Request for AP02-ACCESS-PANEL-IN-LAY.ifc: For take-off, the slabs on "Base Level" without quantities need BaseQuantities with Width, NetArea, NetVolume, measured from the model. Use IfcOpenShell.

First a look at what the model holds.

```python
import ifcopenshell
import ifcopenshell.util.element
import ifcopenshell.util.unit

model = ifcopenshell.open("AP02-ACCESS-PANEL-IN-LAY.ifc")
print(model.schema)
for unit_type in ("LENGTHUNIT", "AREAUNIT", "VOLUMEUNIT"):
    print(unit_type, ifcopenshell.util.unit.calculate_unit_scale(model, unit_type))
storey = next(s for s in model.by_type("IfcBuildingStorey") if s.Name == "Base Level")
slabs = [e for e in ifcopenshell.util.element.get_decomposition(storey) if e.is_a("IfcSlab")]
for e in sorted(slabs, key=lambda e: e.id()):
    print(e.id(), e.is_a(), e.Name, list(ifcopenshell.util.element.get_psets(e, qtos_only=True)), sep=" | ")
```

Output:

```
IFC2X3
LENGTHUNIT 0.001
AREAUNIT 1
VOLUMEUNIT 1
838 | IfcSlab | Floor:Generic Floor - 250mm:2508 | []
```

```python
import ifcopenshell
import ifcopenshell.api.pset
import ifcopenshell.geom
import ifcopenshell.util.element
import ifcopenshell.util.shape
import ifcopenshell.util.unit

model = ifcopenshell.open("AP02-ACCESS-PANEL-IN-LAY.ifc")
unit_scale = ifcopenshell.util.unit.calculate_unit_scale(model)
area_scale = ifcopenshell.util.unit.calculate_unit_scale(model, "AREAUNIT")
volume_scale = ifcopenshell.util.unit.calculate_unit_scale(model, "VOLUMEUNIT")
settings = ifcopenshell.geom.settings()

storey = next(s for s in model.by_type("IfcBuildingStorey") if s.Name == "Base Level")
slabs = [e for e in ifcopenshell.util.element.get_decomposition(storey) if e.is_a("IfcSlab")]

for e in sorted(slabs, key=lambda e: e.id()):
    if ifcopenshell.util.element.get_psets(e, qtos_only=True, should_inherit=False):
        continue
    # Geometry comes back in metres, in the element's own axes.
    shape = ifcopenshell.geom.create_shape(settings, e)
    values = {
        "Width": ifcopenshell.util.shape.get_z(shape.geometry) / unit_scale,
        "NetArea": ifcopenshell.util.shape.get_footprint_area(shape.geometry) / area_scale,
        "NetVolume": ifcopenshell.util.shape.get_volume(shape.geometry) / volume_scale,
    }
    qto = ifcopenshell.api.pset.add_qto(model, product=e, name="BaseQuantities")
    ifcopenshell.api.pset.edit_qto(model, qto=qto, properties=values)
    print(e.id(), {k: round(v, 3) for k, v in values.items()})

model.write("AP02-ACCESS-PANEL-IN-LAY_updated.ifc")
```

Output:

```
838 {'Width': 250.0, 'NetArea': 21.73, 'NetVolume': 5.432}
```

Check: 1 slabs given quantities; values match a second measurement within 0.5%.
